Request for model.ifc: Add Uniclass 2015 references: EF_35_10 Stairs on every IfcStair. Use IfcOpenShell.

First a look at what the model holds.

```python
import ifcopenshell

model = ifcopenshell.open("model.ifc")
print(model.schema)
print("classifications:", [c.Name for c in model.by_type("IfcClassification")])
for ifc_class in ("IfcDoor", "IfcRoof", "IfcStair", "IfcWall", "IfcWindow"):
    print(ifc_class, len(model.by_type(ifc_class)))
```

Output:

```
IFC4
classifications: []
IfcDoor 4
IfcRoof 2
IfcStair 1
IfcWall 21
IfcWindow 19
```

```python
import ifcopenshell
import ifcopenshell.api.classification

model = ifcopenshell.open("model.ifc")

system = ifcopenshell.api.classification.add_classification(model, classification="Uniclass 2015")

codes = {
    "IfcStair": ("EF_35_10", "Stairs"),
}
for ifc_class, (code, name) in codes.items():
    products = model.by_type(ifc_class)
    ifcopenshell.api.classification.add_reference(
        model, products=products, classification=system, identification=code, name=name
    )
    print(code, len(products))

model.write("model_edited.ifc")
```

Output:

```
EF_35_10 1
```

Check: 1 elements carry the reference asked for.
